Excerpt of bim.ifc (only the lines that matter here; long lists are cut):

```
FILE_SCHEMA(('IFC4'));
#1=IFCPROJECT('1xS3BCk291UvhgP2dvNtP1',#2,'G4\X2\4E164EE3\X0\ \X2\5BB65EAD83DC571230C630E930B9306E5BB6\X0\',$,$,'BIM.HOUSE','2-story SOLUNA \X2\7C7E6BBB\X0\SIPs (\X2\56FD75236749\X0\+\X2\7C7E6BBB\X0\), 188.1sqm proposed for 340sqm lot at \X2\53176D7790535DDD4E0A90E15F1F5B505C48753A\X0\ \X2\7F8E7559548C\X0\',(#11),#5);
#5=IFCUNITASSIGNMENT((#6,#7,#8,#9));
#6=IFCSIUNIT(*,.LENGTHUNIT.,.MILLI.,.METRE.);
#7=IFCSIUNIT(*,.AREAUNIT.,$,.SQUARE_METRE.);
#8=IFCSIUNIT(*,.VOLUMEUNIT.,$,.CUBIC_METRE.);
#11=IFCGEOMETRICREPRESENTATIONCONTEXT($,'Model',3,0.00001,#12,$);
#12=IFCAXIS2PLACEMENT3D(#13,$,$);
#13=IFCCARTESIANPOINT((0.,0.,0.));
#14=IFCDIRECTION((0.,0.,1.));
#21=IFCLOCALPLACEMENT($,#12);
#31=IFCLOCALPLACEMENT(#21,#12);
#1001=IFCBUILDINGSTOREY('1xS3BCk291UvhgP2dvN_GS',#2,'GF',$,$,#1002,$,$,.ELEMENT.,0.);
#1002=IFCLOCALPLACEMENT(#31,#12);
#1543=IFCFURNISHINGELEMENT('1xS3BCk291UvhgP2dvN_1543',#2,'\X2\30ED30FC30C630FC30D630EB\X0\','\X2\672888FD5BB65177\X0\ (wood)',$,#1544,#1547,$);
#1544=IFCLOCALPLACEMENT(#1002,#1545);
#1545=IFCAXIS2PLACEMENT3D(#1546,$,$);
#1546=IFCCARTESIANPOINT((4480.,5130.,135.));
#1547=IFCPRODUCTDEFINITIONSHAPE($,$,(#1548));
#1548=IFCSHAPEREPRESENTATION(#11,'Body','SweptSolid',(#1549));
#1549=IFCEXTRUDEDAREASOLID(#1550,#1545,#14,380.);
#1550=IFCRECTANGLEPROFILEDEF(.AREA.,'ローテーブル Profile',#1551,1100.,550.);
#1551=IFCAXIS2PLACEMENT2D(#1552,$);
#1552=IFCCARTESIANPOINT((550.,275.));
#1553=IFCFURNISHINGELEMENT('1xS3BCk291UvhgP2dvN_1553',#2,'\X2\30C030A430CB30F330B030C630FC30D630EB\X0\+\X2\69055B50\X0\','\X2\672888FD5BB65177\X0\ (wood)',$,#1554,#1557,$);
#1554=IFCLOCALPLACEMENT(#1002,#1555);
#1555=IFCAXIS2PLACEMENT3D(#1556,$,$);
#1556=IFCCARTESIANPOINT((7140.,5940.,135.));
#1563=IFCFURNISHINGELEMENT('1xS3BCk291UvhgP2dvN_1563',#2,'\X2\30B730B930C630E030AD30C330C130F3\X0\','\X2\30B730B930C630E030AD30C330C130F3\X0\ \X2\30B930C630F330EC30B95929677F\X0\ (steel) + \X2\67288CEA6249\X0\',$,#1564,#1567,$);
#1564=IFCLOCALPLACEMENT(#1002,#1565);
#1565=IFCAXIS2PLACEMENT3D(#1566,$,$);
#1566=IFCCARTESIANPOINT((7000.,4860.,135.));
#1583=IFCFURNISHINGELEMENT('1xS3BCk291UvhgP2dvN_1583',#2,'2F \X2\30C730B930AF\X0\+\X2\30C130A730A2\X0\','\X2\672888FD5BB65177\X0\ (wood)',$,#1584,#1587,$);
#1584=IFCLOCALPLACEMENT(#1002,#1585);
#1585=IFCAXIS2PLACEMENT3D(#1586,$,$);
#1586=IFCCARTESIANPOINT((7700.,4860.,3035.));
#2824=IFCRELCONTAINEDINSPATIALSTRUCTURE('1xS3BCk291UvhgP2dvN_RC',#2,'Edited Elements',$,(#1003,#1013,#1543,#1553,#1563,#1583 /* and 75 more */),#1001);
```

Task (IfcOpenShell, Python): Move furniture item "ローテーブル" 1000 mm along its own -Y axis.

```python
import ifcopenshell
import ifcopenshell.api.geometry
import ifcopenshell.util.placement

model = ifcopenshell.open("bim.ifc")

item = model.by_id(1543)
matrix = ifcopenshell.util.placement.get_local_placement(item.ObjectPlacement)
matrix[:3, 3] -= matrix[:3, 1] * 1000.0
ifcopenshell.api.geometry.edit_object_placement(model, product=item, matrix=matrix, is_si=False)

print(ifcopenshell.util.placement.get_local_placement(item.ObjectPlacement).round(3) + 0.0)

model.write("bim_edited.ifc")
```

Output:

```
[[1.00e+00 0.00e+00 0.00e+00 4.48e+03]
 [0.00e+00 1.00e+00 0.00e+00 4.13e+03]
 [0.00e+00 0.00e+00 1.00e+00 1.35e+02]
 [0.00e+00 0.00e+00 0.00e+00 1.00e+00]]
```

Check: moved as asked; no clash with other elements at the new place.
